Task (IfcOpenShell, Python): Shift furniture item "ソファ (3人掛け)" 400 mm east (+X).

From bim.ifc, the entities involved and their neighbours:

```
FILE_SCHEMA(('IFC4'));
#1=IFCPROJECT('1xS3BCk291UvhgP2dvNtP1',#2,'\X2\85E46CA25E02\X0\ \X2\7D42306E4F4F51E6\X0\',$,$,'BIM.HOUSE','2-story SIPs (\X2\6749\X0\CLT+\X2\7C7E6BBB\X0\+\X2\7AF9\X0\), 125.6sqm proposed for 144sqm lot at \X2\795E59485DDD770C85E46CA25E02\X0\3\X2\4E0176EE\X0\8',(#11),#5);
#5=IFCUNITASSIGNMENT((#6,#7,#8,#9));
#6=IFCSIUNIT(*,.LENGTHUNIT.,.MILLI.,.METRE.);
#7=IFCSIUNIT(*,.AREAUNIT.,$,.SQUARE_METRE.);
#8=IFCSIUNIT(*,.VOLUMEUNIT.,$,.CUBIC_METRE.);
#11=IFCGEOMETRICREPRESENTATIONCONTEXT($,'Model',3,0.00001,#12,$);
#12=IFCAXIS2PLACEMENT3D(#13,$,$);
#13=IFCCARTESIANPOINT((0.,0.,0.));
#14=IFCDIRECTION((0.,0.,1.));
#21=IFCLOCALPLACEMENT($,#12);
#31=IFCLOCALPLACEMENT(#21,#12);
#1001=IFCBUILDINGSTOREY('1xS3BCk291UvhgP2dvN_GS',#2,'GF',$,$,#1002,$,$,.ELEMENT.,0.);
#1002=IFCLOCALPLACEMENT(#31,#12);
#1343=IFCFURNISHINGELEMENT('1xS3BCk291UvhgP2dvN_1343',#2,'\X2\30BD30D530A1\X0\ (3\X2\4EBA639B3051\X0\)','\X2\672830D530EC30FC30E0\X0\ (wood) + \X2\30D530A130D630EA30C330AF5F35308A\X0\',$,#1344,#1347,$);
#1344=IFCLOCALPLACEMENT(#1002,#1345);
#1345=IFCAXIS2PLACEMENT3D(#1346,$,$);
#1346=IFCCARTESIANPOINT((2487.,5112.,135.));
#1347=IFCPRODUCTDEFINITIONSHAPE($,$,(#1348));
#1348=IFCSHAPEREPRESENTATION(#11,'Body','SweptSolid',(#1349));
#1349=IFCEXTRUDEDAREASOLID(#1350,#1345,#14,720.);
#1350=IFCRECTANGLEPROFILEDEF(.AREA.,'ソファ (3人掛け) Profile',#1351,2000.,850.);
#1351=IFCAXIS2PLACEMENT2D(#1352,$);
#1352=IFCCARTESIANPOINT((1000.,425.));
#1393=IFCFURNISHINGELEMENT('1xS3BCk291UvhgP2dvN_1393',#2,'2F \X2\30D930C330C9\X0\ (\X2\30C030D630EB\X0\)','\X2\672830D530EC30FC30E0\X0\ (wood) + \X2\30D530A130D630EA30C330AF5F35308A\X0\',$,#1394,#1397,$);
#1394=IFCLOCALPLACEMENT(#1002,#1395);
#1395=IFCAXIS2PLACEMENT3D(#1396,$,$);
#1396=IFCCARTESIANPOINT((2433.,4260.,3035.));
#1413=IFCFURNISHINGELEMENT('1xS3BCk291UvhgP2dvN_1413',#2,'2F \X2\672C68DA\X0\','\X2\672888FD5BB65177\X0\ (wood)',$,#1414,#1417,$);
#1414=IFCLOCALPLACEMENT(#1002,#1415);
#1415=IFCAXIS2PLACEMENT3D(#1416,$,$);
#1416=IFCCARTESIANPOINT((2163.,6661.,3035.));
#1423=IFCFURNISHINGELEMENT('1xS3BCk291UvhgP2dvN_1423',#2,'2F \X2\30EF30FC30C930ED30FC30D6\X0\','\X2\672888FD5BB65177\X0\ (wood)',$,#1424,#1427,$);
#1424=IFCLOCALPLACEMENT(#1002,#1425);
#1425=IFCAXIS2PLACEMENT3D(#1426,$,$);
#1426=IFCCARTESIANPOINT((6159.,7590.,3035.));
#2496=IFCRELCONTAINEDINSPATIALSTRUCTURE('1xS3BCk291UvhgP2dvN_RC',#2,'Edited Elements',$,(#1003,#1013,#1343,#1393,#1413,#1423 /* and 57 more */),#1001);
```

```python
import ifcopenshell
import ifcopenshell.api.geometry
import ifcopenshell.util.placement
import ifcopenshell.util.unit

model = ifcopenshell.open("bim.ifc")
unit_scale = ifcopenshell.util.unit.calculate_unit_scale(model)

item = model.by_guid("1xS3BCk291UvhgP2dvN_1343")
matrix = ifcopenshell.util.placement.get_local_placement(item.ObjectPlacement)
matrix[0, 3] += 0.4 / unit_scale
ifcopenshell.api.geometry.edit_object_placement(model, product=item, matrix=matrix, is_si=False)

print(ifcopenshell.util.placement.get_local_placement(item.ObjectPlacement).round(3) + 0.0)

model.write("bim_edited.ifc")
```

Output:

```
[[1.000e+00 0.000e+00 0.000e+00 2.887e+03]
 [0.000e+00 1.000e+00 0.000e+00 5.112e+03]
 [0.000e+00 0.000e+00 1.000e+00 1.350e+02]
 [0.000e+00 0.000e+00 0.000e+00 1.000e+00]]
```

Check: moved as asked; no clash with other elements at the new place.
